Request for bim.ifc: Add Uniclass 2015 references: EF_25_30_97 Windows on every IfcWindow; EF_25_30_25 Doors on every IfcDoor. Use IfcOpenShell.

First a look at what the model holds.

```python
import ifcopenshell

model = ifcopenshell.open("bim.ifc")
print(model.schema)
print("classifications:", [c.Name for c in model.by_type("IfcClassification")])
for ifc_class in ("IfcDoor", "IfcRoof", "IfcStair", "IfcWall", "IfcWindow"):
    print(ifc_class, len(model.by_type(ifc_class)))
```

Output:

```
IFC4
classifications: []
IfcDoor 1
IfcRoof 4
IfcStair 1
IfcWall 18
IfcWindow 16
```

```python
import ifcopenshell
import ifcopenshell.api.classification

model = ifcopenshell.open("bim.ifc")

system = ifcopenshell.api.classification.add_classification(model, classification="Uniclass 2015")

codes = {
    "IfcWindow": ("EF_25_30_97", "Windows"),
    "IfcDoor": ("EF_25_30_25", "Doors"),
}
for ifc_class, (code, name) in codes.items():
    products = model.by_type(ifc_class)
    ifcopenshell.api.classification.add_reference(
        model, products=products, classification=system, identification=code, name=name
    )
    print(code, len(products))

model.write("bim_updated.ifc")
```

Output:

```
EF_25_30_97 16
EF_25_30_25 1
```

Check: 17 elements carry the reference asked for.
